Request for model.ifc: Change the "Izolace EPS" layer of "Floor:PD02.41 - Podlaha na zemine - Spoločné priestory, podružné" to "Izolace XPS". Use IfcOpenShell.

First a look at what the model holds.

```python
import ifcopenshell
import ifcopenshell.util.element

model = ifcopenshell.open("model.ifc")
print(model.schema)
for layer_set in model.by_type("IfcMaterialLayerSet"):
    if layer_set.LayerSetName == "Floor:PD02.41 - Podlaha na zemine - Spoločné priestory, podružné":
        for layer in layer_set.MaterialLayers:
            print(layer.id(), layer.Material and layer.Material.Name, layer.LayerThickness, sep=" | ")
        print(len(ifcopenshell.util.element.get_elements_by_material(model, layer_set)), "elements and types use it")
print(sorted(m.Name for m in model.by_type("IfcMaterial") if m.Name)[:60])
```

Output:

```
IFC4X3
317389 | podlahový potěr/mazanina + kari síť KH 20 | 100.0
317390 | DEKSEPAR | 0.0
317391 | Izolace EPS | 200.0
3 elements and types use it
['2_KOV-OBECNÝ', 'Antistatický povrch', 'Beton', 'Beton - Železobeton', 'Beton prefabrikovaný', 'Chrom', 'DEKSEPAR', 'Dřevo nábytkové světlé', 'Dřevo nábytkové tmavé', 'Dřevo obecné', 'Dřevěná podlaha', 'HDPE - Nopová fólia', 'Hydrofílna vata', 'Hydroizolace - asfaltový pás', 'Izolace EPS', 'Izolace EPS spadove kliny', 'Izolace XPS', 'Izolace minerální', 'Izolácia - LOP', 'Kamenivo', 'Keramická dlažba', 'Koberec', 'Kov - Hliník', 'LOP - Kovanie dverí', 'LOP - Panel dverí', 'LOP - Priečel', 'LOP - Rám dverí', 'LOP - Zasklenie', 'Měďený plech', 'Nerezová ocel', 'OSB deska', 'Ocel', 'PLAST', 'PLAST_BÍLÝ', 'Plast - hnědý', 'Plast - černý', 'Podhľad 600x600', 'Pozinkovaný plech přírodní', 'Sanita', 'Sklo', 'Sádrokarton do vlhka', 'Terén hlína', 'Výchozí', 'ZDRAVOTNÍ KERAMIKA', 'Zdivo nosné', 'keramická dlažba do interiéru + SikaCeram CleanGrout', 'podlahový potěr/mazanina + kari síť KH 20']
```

```python
import ifcopenshell
import ifcopenshell.api.material

model = ifcopenshell.open("model.ifc")

layer_set = next(s for s in model.by_type("IfcMaterialLayerSet") if s.LayerSetName == "Floor:PD02.41 - Podlaha na zemine - Spoločné priestory, podružné")
layer = next(l for l in layer_set.MaterialLayers if l.Material and l.Material.Name == "Izolace EPS")
material = next(m for m in model.by_type("IfcMaterial") if m.Name == "Izolace XPS")

# Point this one layer at the other material; renaming the old one would change it everywhere.
ifcopenshell.api.material.edit_layer(model, layer=layer, attributes={"Name": material.Name}, material=material)

print([l.Material.Name if l.Material else None for l in layer_set.MaterialLayers])

model.write("model_rev.ifc")
```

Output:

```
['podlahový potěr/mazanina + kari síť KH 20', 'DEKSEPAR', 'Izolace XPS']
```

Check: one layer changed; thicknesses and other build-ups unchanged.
